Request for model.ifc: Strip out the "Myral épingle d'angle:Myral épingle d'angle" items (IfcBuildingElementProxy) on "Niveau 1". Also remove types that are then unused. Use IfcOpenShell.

First a look at what the model holds.

```python
import ifcopenshell
import ifcopenshell.util.element

model = ifcopenshell.open("model.ifc")
print(model.schema)
storey = next(s for s in model.by_type("IfcBuildingStorey") if s.Name == "Niveau 1")
proxies = [e for e in ifcopenshell.util.element.get_decomposition(storey) if e.is_a("IfcBuildingElementProxy")]
seen = {}
for e in proxies:
    element_type = ifcopenshell.util.element.get_type(e)
    name = element_type.Name if element_type not in (None, e) else None
    seen[name] = seen.get(name, 0) + 1
for name, count in sorted(seen.items(), key=str):
    print(count, "x", name)
```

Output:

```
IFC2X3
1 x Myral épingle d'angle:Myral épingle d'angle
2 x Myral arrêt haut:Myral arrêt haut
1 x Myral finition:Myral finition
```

```python
import ifcopenshell
import ifcopenshell.api.root
import ifcopenshell.util.element

model = ifcopenshell.open("model.ifc")

storey = next(s for s in model.by_type("IfcBuildingStorey") if s.Name == "Niveau 1")
proxies = [e for e in ifcopenshell.util.element.get_decomposition(storey) if e.is_a("IfcBuildingElementProxy")]
targets = [e for e in proxies if (t := ifcopenshell.util.element.get_type(e)) not in (None, e) and t.Name == "Myral épingle d'angle:Myral épingle d'angle"]
types = {ifcopenshell.util.element.get_type(e) for e in targets} - {None, *targets}

for e in targets:
    ifcopenshell.api.root.remove_product(model, product=e)
print(len(targets), "removed")

unused = [t for t in types if not ifcopenshell.util.element.get_types(t)]
for t in unused:
    ifcopenshell.api.root.remove_product(model, product=t)
print(len(unused), "unused types removed")

model.write("model-out.ifc")
```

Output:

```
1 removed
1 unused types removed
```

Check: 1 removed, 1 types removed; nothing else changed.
